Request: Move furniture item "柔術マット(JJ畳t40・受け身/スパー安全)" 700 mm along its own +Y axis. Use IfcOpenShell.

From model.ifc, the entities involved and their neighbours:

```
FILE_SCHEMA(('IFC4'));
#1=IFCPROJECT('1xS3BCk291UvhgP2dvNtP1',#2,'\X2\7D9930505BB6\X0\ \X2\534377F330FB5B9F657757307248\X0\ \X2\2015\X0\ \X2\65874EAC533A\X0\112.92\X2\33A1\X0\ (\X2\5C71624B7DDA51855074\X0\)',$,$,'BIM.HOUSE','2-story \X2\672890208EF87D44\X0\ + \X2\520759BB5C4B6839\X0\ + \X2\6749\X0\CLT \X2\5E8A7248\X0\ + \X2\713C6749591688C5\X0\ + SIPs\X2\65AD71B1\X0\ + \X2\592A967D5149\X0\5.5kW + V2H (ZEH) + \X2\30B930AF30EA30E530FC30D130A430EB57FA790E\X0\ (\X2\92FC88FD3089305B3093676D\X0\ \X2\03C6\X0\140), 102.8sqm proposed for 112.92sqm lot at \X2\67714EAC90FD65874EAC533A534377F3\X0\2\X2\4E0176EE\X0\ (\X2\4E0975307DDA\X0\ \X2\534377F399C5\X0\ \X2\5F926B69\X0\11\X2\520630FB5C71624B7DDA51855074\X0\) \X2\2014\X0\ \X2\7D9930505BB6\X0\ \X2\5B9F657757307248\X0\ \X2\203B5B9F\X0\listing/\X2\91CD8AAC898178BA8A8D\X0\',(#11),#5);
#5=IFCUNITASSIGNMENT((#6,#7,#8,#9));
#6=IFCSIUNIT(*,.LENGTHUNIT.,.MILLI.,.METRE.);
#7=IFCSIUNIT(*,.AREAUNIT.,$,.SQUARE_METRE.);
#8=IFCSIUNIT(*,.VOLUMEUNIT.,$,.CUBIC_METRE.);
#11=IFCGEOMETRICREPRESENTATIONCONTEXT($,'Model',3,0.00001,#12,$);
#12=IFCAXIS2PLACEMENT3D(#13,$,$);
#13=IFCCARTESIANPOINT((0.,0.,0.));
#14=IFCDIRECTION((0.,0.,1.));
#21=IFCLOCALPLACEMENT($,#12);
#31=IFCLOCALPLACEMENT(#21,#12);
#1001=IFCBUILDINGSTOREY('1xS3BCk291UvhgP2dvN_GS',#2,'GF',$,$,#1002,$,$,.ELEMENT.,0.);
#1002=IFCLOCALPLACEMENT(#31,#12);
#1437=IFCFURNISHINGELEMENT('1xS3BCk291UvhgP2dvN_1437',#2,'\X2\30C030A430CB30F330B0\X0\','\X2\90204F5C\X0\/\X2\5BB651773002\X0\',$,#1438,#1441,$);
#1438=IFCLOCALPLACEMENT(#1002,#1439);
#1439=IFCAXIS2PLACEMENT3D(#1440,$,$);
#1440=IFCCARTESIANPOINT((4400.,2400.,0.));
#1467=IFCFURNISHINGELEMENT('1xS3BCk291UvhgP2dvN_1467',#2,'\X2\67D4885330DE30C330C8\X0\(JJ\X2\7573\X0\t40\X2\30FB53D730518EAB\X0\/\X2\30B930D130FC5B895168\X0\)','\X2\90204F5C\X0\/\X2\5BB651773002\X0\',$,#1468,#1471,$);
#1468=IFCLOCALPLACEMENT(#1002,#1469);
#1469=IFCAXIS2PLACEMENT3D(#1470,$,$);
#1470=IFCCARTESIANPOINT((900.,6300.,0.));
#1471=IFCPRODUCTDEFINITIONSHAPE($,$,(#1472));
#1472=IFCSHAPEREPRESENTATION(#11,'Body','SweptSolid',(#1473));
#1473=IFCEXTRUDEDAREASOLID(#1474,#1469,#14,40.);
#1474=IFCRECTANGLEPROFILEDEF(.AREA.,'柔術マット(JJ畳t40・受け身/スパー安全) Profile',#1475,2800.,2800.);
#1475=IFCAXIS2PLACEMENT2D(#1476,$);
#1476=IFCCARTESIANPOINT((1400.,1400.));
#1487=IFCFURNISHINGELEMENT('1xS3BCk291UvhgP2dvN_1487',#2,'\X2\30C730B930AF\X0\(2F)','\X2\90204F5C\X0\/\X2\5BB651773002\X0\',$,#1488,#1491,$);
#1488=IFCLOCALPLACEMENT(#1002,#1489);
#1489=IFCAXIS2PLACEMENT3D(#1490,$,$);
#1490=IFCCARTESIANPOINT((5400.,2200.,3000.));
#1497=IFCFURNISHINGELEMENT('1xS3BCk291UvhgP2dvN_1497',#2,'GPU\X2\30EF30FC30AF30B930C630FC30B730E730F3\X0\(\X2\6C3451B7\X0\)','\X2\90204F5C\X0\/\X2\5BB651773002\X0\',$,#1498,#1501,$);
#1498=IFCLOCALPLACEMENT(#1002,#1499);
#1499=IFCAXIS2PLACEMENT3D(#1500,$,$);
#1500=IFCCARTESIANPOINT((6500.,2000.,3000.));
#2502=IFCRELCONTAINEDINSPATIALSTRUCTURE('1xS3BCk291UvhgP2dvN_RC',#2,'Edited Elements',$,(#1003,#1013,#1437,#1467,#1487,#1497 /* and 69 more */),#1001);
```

```python
import ifcopenshell
import ifcopenshell.api.geometry
import ifcopenshell.util.placement
import ifcopenshell.util.unit

model = ifcopenshell.open("model.ifc")
unit_scale = ifcopenshell.util.unit.calculate_unit_scale(model)

item = model.by_guid("1xS3BCk291UvhgP2dvN_1467")
matrix = ifcopenshell.util.placement.get_local_placement(item.ObjectPlacement)
matrix[:3, 3] += matrix[:3, 1] * 0.7 / unit_scale
ifcopenshell.api.geometry.edit_object_placement(model, product=item, matrix=matrix, is_si=False)

print(ifcopenshell.util.placement.get_local_placement(item.ObjectPlacement).round(3) + 0.0)

model.write("model_rev.ifc")
```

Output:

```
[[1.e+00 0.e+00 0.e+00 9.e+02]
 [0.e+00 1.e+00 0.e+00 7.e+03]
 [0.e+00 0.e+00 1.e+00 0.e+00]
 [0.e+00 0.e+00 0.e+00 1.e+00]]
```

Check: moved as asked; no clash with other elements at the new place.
